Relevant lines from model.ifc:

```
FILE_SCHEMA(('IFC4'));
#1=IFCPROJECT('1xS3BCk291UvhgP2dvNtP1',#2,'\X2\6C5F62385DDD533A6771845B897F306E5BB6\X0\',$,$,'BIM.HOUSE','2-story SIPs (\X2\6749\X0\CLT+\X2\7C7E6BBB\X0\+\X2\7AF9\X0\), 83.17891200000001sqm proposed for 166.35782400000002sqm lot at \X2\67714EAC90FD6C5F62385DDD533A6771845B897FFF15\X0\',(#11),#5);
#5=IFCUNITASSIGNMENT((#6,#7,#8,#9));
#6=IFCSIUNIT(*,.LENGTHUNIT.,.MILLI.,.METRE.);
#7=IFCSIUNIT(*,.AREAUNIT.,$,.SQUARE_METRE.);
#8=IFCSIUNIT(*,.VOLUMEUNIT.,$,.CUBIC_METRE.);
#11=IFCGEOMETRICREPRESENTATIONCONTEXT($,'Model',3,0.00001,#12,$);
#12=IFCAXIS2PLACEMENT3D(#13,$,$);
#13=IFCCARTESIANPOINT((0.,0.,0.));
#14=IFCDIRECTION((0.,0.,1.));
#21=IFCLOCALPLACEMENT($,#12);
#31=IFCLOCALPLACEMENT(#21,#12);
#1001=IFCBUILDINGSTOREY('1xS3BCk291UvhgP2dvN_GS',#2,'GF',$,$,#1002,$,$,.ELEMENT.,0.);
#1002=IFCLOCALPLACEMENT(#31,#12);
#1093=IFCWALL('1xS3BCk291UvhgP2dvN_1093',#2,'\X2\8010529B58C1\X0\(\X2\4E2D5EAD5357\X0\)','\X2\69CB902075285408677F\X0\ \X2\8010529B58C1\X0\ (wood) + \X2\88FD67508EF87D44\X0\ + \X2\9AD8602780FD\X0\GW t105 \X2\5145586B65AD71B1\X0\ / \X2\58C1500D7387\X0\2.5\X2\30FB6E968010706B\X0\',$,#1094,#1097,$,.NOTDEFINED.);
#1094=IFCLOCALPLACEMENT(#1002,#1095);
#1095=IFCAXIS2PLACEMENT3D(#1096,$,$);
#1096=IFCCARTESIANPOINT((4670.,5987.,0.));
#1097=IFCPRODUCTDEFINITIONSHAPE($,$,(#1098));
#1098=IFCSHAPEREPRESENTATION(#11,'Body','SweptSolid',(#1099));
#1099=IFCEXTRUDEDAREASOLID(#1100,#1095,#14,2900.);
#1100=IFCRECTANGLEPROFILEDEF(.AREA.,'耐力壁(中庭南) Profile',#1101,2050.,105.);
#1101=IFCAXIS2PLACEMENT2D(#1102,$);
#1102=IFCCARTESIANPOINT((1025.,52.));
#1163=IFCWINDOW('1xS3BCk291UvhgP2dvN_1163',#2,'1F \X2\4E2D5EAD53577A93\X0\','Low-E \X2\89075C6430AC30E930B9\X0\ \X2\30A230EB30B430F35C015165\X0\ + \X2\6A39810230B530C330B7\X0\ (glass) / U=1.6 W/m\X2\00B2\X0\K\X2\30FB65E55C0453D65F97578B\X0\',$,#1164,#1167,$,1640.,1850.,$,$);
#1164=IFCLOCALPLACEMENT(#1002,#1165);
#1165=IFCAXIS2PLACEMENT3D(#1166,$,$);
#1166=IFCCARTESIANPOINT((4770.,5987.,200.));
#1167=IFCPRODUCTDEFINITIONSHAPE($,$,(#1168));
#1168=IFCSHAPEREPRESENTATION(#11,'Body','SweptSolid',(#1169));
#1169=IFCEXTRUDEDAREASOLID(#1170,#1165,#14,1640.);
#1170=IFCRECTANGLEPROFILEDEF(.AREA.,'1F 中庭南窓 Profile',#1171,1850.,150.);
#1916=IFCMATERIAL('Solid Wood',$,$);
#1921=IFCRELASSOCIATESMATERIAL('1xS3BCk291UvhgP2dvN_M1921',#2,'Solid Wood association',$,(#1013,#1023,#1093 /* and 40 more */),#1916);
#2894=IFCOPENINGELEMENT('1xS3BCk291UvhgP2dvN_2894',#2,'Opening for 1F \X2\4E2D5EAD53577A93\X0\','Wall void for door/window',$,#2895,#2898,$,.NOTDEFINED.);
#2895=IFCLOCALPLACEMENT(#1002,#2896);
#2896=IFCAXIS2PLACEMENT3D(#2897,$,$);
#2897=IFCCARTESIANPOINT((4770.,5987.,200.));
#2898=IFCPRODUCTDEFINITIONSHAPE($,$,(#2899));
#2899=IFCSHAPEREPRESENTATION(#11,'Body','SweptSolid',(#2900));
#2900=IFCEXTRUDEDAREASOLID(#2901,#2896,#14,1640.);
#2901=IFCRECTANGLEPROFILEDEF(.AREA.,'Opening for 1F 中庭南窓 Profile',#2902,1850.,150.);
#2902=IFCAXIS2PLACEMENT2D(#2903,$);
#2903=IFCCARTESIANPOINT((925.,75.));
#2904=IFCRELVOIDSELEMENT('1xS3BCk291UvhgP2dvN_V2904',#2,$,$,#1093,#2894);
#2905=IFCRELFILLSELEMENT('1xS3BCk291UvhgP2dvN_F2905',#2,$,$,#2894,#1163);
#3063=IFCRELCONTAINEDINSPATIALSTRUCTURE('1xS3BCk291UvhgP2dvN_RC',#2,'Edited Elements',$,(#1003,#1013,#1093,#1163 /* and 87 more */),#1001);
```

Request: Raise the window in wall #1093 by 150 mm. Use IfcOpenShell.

```python
import numpy as np
import ifcopenshell
import ifcopenshell.api.geometry
import ifcopenshell.util.placement
import ifcopenshell.util.unit

model = ifcopenshell.open("model.ifc")
unit_scale = ifcopenshell.util.unit.calculate_unit_scale(model)

window = model.by_id(1163)
opening = window.FillsVoids[0].RelatingOpeningElement
dz = 150.0

shift = np.array([0.0, 0.0, dz])
# The window is not placed relative to its opening, so move both.
for product in (opening, window):
    matrix = ifcopenshell.util.placement.get_local_placement(product.ObjectPlacement)
    matrix[:3, 3] += shift
    ifcopenshell.api.geometry.edit_object_placement(model, product=product, matrix=matrix, is_si=False)

print(f"moved by {dz * unit_scale:+.3f} m")

model.write("model_v2.ifc")
```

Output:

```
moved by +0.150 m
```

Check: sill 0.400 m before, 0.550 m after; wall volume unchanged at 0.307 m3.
